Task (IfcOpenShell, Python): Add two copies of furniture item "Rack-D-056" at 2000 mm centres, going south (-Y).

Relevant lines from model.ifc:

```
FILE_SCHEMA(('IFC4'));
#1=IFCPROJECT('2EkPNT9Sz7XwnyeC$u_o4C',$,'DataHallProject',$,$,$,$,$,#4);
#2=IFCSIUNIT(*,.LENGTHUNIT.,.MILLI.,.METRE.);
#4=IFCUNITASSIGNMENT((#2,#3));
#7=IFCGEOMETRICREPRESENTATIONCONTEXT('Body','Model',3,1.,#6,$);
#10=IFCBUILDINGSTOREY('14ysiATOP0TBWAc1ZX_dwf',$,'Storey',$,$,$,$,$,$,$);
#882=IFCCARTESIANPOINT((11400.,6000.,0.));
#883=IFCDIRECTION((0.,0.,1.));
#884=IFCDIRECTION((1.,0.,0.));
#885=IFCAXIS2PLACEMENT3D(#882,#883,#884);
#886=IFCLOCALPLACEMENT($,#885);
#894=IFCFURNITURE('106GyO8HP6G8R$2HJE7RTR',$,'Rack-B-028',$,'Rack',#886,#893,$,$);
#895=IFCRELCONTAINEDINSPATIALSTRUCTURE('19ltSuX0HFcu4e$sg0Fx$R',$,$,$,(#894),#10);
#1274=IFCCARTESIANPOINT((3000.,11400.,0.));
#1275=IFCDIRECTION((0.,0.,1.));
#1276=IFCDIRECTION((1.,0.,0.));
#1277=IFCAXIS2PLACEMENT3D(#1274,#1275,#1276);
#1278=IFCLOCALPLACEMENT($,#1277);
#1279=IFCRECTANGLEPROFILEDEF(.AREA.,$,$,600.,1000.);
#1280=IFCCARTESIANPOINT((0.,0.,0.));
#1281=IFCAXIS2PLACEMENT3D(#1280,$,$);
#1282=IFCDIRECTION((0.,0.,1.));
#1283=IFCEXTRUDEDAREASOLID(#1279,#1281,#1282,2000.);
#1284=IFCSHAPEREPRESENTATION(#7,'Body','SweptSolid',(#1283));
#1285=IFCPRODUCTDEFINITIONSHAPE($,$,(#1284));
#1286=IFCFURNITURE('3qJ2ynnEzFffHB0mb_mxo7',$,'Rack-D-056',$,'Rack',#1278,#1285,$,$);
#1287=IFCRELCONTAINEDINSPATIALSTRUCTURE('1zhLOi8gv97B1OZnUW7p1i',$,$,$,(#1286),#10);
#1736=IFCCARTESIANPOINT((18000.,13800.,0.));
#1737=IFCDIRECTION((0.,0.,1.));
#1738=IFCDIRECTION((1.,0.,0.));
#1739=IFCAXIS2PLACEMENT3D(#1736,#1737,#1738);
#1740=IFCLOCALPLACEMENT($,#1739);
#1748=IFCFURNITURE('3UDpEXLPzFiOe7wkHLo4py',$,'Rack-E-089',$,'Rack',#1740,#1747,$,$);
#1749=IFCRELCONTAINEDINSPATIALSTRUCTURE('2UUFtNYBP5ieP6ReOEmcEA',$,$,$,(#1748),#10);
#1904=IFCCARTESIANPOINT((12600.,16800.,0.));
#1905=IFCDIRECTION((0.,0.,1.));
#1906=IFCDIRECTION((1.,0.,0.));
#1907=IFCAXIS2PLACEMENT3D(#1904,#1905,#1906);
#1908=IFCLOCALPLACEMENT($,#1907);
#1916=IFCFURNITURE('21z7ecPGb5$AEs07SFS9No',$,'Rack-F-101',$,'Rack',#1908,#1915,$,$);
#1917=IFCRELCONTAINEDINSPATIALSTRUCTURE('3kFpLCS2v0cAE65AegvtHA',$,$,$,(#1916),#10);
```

```python
import numpy as np
import ifcopenshell
import ifcopenshell.api.geometry
import ifcopenshell.api.root
import ifcopenshell.util.element
import ifcopenshell.util.placement

model = ifcopenshell.open("model.ifc")

source = model.by_id(1286)
base = ifcopenshell.util.placement.get_local_placement(source.ObjectPlacement)
step = np.array([0.0, -1.0, 0.0]) * 2000.0

for i in range(1, 3):
    copy = ifcopenshell.api.root.copy_class(model, product=source)
    copy.Representation = ifcopenshell.util.element.copy_deep(
        model, source.Representation, exclude=["IfcGeometricRepresentationContext", "IfcRepresentationMap"]
    )
    matrix = base.copy()
    matrix[:3, 3] += i * step
    print("added at", matrix[:3, 3].round(3) + 0.0)
    ifcopenshell.api.geometry.edit_object_placement(model, product=copy, matrix=matrix, is_si=False)

model.write("model_updated.ifc")
```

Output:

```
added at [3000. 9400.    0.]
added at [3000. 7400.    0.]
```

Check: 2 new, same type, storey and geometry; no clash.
